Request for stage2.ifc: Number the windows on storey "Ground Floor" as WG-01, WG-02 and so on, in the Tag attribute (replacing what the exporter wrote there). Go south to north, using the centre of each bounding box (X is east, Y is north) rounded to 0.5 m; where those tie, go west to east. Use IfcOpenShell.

First a look at what the model holds.

```python
import ifcopenshell
import ifcopenshell.util.element
import ifcopenshell.util.placement

model = ifcopenshell.open("stage2.ifc")
print(model.schema)
storey = next(s for s in model.by_type("IfcBuildingStorey") if s.Name == "Ground Floor")
windows = [e for e in ifcopenshell.util.element.get_decomposition(storey) if e.is_a("IfcWindow")]
for e in sorted(windows, key=lambda e: e.id()):
    origin = ifcopenshell.util.placement.get_local_placement(e.ObjectPlacement)[:3, 3]
    print(e.id(), e.Tag, e.Name, origin.round(2) + 0.0, sep=" | ")
```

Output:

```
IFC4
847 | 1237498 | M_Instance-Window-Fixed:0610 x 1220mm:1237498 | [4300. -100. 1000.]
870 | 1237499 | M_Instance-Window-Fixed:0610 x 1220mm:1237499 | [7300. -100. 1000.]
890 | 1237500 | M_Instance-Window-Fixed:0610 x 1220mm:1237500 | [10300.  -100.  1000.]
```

```python
import ifcopenshell
import ifcopenshell.geom
import ifcopenshell.util.element
import ifcopenshell.util.shape

model = ifcopenshell.open("stage2.ifc")
settings = ifcopenshell.geom.settings()
settings.set("use-world-coords", True)


def centre(element):
    shape = ifcopenshell.geom.create_shape(settings, element)
    return ifcopenshell.util.shape.get_bbox_centroid(shape.geometry)


storey = next(s for s in model.by_type("IfcBuildingStorey") if s.Name == "Ground Floor")
windows = [e for e in ifcopenshell.util.element.get_decomposition(storey) if e.is_a("IfcWindow")]

# Insertion points can sit at a corner or the storey origin, so sort by the geometry (in metres).
centres = {e: centre(e) for e in windows}
windows.sort(key=lambda e: (round(centres[e][1] / 0.5), centres[e][0]))

for i, e in enumerate(windows, start=1):
    number = f"WG-{i:02d}"
    e.Tag = number
    print(e.id(), number)

model.write("stage2-out.ifc")
```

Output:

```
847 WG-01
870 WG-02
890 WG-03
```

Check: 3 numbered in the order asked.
